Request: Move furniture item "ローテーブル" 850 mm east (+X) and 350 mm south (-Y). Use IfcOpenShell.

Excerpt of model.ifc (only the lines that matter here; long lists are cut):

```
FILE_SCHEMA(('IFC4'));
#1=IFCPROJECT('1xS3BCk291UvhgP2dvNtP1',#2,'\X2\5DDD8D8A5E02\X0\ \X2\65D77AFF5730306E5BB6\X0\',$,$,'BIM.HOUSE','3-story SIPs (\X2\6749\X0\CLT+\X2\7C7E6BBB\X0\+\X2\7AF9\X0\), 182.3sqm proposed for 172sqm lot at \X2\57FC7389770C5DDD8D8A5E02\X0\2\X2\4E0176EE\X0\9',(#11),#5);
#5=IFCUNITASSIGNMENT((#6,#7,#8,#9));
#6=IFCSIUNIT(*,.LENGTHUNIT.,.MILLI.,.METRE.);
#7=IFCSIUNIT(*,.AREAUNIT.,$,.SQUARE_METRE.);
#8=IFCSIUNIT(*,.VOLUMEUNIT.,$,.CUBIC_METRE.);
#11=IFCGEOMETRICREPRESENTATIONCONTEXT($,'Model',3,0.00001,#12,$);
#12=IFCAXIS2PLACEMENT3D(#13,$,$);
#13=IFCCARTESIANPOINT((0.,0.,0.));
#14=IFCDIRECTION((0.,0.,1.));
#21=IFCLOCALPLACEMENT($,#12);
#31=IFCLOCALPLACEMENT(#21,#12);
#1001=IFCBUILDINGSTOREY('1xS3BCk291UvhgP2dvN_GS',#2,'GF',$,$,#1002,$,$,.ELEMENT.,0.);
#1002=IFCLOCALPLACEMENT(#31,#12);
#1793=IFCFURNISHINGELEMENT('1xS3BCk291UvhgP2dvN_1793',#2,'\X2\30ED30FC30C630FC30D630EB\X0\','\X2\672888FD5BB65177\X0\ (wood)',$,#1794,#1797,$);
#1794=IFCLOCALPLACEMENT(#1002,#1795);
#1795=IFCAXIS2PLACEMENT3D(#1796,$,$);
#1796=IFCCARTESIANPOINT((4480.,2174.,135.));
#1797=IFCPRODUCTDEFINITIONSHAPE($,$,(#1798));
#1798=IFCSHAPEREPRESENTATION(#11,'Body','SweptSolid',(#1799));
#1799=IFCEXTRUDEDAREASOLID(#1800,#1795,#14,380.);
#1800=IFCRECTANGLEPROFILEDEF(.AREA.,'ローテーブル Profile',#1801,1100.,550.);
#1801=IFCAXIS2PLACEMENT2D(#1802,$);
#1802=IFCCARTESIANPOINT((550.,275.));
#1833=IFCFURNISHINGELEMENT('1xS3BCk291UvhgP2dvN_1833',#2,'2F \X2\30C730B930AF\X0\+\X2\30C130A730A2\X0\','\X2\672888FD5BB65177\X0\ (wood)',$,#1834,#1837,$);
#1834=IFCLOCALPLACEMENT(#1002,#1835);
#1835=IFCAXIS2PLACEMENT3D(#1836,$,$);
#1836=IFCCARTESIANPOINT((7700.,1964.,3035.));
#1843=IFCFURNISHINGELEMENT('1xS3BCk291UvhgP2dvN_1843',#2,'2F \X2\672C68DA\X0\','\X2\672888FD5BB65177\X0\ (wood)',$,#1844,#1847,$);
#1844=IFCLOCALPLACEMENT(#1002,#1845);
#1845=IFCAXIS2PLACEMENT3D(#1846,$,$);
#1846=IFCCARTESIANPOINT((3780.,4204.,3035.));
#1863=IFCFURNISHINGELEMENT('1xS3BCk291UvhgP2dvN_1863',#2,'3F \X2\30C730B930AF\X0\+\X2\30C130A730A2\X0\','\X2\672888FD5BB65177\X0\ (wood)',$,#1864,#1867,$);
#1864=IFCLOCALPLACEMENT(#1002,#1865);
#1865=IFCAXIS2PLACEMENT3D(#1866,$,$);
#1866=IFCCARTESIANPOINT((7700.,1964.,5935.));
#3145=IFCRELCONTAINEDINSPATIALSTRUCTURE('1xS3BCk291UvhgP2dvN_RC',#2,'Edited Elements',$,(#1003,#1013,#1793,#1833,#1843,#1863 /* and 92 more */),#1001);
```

```python
import ifcopenshell
import ifcopenshell.api.geometry
import ifcopenshell.util.placement
import ifcopenshell.util.unit

model = ifcopenshell.open("model.ifc")
unit_scale = ifcopenshell.util.unit.calculate_unit_scale(model)

item = model.by_id(1793)
matrix = ifcopenshell.util.placement.get_local_placement(item.ObjectPlacement)
matrix[0, 3] += 0.85 / unit_scale
matrix[1, 3] -= 0.35 / unit_scale
ifcopenshell.api.geometry.edit_object_placement(model, product=item, matrix=matrix, is_si=False)

print(ifcopenshell.util.placement.get_local_placement(item.ObjectPlacement).round(3) + 0.0)

model.write("model_rev.ifc")
```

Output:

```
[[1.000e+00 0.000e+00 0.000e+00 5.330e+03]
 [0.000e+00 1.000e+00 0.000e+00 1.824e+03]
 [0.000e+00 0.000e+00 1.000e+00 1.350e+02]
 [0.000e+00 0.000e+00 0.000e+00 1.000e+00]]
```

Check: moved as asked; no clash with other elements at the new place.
